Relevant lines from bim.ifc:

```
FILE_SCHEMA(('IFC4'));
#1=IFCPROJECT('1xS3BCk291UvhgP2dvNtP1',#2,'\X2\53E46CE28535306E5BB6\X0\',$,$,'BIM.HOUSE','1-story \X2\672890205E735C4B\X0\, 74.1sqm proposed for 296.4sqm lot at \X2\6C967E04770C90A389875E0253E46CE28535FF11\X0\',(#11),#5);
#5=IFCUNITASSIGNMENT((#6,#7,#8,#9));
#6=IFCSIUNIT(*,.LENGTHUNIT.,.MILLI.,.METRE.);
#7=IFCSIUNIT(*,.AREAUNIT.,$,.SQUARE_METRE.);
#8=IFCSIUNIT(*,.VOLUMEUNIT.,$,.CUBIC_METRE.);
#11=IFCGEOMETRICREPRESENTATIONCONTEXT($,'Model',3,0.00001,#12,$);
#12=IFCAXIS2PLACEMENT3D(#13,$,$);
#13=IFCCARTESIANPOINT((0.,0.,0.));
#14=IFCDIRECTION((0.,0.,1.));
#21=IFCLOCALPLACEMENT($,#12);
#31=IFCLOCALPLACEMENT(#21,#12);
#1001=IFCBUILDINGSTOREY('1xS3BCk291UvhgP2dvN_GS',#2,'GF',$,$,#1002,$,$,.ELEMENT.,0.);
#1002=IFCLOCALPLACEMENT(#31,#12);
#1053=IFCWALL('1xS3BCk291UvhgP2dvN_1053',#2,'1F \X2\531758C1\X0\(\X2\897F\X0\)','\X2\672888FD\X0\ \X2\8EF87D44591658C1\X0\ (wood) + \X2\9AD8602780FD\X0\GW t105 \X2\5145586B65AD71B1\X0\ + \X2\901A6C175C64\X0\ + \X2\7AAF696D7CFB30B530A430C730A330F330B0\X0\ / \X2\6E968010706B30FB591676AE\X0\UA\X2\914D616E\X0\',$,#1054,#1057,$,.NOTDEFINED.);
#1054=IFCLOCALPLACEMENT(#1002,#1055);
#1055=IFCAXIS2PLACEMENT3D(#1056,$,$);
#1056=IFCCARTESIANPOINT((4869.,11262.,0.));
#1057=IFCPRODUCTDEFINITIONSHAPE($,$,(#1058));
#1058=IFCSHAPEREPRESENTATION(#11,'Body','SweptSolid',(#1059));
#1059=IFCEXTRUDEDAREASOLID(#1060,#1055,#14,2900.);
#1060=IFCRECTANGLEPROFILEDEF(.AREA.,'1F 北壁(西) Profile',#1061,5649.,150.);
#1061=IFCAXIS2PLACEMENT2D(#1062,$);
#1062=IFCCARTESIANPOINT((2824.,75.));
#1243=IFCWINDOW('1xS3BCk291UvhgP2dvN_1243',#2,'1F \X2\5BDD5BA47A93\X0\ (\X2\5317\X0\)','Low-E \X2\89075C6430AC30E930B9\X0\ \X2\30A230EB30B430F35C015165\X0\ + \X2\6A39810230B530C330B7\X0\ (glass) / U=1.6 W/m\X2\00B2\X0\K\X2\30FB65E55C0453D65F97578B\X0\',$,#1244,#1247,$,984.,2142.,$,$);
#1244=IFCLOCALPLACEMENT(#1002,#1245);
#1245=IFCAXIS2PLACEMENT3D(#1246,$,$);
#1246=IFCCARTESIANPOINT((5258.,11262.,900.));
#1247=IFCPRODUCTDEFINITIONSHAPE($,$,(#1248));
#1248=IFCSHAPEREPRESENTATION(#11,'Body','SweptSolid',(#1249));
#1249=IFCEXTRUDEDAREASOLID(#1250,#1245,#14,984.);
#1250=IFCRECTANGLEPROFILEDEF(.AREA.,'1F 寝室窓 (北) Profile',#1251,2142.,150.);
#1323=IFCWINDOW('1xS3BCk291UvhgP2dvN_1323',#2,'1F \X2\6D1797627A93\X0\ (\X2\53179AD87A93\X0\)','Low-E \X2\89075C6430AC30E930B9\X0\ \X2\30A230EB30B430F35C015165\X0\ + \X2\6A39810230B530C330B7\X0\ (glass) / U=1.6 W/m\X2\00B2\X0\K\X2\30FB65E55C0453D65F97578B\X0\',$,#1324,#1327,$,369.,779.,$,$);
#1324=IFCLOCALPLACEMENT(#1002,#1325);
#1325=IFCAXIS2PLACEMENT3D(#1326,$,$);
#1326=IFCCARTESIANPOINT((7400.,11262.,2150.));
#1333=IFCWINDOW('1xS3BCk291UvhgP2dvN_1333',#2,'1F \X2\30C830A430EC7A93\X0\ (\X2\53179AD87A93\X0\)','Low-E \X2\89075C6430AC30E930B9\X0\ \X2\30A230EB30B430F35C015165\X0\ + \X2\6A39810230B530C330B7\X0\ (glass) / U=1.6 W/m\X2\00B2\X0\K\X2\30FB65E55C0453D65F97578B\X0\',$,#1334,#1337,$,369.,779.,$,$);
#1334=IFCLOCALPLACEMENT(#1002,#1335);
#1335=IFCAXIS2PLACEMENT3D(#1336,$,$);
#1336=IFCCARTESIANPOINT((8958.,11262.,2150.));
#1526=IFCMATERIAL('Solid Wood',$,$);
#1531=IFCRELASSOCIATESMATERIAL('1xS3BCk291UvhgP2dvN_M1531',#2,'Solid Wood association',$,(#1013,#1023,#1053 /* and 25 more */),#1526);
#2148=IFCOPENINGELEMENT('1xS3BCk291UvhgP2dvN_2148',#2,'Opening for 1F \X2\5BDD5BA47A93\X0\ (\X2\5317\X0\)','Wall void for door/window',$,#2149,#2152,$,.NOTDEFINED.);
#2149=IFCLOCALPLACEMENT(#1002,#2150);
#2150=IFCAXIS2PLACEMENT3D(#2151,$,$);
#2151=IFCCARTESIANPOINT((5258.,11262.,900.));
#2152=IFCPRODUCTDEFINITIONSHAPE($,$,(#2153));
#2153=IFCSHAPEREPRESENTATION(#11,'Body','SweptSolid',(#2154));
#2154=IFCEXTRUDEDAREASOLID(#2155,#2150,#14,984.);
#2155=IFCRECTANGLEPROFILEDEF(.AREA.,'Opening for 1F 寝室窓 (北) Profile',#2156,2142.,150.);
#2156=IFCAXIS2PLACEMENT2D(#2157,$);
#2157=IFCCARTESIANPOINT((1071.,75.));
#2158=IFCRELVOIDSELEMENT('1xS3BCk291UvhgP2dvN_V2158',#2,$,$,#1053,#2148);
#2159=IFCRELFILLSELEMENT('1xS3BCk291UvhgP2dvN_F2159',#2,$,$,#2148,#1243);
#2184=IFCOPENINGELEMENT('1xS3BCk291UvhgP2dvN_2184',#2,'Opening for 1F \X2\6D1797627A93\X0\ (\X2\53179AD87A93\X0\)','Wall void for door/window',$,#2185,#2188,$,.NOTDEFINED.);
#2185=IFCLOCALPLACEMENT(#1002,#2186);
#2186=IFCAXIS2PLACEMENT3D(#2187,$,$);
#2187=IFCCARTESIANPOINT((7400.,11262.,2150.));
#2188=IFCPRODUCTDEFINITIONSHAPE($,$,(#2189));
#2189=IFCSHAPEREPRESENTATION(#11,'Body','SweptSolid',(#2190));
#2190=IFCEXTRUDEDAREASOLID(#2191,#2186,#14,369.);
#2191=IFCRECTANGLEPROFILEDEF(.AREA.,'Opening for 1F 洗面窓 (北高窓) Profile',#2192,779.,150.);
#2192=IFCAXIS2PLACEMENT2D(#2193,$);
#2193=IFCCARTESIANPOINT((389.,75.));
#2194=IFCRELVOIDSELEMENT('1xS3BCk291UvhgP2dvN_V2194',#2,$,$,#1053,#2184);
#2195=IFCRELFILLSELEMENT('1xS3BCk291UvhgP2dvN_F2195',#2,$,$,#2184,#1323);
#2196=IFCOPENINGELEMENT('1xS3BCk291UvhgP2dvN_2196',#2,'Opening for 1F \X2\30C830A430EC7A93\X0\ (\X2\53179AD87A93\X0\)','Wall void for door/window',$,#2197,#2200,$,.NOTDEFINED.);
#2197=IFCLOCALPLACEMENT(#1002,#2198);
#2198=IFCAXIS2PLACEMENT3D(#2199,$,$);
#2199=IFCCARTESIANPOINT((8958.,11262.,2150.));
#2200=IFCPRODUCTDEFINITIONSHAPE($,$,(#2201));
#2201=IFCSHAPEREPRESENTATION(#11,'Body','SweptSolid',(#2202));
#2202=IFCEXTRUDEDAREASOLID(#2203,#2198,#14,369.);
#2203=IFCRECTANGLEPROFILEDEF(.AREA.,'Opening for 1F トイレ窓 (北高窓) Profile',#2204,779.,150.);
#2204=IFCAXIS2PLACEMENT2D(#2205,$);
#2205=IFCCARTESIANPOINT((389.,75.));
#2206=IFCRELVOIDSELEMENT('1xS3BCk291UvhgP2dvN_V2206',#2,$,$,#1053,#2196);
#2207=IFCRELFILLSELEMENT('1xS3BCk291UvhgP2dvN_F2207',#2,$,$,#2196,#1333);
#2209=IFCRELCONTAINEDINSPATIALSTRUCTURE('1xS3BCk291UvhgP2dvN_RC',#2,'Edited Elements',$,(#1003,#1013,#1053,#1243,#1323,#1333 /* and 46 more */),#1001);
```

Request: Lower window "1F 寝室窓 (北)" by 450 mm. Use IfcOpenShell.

```python
import numpy as np
import ifcopenshell
import ifcopenshell.api.geometry
import ifcopenshell.util.placement
import ifcopenshell.util.unit

model = ifcopenshell.open("bim.ifc")
unit_scale = ifcopenshell.util.unit.calculate_unit_scale(model)

window = model.by_guid("1xS3BCk291UvhgP2dvN_1243")
opening = window.FillsVoids[0].RelatingOpeningElement
dz = -0.45 / unit_scale

shift = np.array([0.0, 0.0, dz])
# The window is not placed relative to its opening, so move both.
for product in (opening, window):
    matrix = ifcopenshell.util.placement.get_local_placement(product.ObjectPlacement)
    matrix[:3, 3] += shift
    ifcopenshell.api.geometry.edit_object_placement(model, product=product, matrix=matrix, is_si=False)

print(f"moved by {dz * unit_scale:+.3f} m")

model.write("bim-out.ifc")
```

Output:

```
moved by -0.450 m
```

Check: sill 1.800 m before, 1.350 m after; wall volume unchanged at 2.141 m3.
